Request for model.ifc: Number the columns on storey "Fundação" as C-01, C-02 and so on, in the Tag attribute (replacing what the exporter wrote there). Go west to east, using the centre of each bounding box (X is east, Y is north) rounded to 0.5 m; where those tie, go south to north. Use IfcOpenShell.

First a look at what the model holds.

```python
import ifcopenshell
import ifcopenshell.util.element
import ifcopenshell.util.placement

model = ifcopenshell.open("model.ifc")
print(model.schema)
storey = next(s for s in model.by_type("IfcBuildingStorey") if s.Name == "Fundação")
columns = [e for e in ifcopenshell.util.element.get_decomposition(storey) if e.is_a("IfcColumn")]
for e in sorted(columns, key=lambda e: e.id()):
    origin = ifcopenshell.util.placement.get_local_placement(e.ObjectPlacement)[:3, 3]
    print(e.id(), e.Tag, e.Name, origin.round(2) + 0.0, sep=" | ")
```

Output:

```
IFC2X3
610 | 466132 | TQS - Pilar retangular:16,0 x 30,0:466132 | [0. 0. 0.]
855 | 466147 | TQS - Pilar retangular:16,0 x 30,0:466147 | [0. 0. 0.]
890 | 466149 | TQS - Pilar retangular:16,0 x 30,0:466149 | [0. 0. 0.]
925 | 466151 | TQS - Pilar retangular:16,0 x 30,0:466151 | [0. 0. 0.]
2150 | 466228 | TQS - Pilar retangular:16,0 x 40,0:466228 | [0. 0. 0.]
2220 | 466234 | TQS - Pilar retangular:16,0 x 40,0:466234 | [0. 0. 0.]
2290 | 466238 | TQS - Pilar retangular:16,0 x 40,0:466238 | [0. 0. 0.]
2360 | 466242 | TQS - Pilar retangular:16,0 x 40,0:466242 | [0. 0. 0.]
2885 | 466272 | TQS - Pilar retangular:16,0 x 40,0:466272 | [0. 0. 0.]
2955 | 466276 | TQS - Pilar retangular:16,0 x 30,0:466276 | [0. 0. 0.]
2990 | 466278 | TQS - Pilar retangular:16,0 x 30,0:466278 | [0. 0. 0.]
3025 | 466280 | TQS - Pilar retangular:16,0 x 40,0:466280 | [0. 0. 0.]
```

```python
import ifcopenshell
import ifcopenshell.geom
import ifcopenshell.util.element
import ifcopenshell.util.shape

model = ifcopenshell.open("model.ifc")
settings = ifcopenshell.geom.settings()
settings.set("use-world-coords", True)


def centre(element):
    shape = ifcopenshell.geom.create_shape(settings, element)
    return ifcopenshell.util.shape.get_bbox_centroid(shape.geometry)


storey = next(s for s in model.by_type("IfcBuildingStorey") if s.Name == "Fundação")
columns = [e for e in ifcopenshell.util.element.get_decomposition(storey) if e.is_a("IfcColumn")]

# Insertion points can sit at a corner or the storey origin, so sort by the geometry (in metres).
centres = {e: centre(e) for e in columns}
columns.sort(key=lambda e: (round(centres[e][0] / 0.5), centres[e][1]))

for i, e in enumerate(columns, start=1):
    number = f"C-{i:02d}"
    e.Tag = number
    print(e.id(), number)

model.write("model-out.ifc")
```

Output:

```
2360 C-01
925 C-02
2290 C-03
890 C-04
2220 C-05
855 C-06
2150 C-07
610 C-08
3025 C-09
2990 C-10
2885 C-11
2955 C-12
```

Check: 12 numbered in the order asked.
